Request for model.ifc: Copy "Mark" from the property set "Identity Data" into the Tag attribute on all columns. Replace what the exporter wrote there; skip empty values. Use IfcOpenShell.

First a look at what the model holds.

```python
import ifcopenshell
import ifcopenshell.util.element

model = ifcopenshell.open("model.ifc")
print(model.schema)
columns = model.by_type("IfcColumn")
print(len(columns), "columns")
for e in columns[:8]:
    source = ifcopenshell.util.element.get_pset(e, "Identity Data", "Mark")
    target = e.Tag
    print(e.id(), repr(source), repr(target), sep=" | ")
```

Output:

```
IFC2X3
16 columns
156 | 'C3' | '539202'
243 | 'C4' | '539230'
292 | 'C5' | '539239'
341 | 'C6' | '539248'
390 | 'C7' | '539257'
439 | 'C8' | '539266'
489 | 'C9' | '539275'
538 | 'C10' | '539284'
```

```python
import ifcopenshell
import ifcopenshell.util.element

model = ifcopenshell.open("model.ifc")

count = 0
for e in model.by_type("IfcColumn"):
    value = ifcopenshell.util.element.get_pset(e, "Identity Data", "Mark")
    current = e.Tag
    if not value or not value.strip() or current == value:
        continue
    e.Tag = value
    count += 1

print(count, "columns updated")

model.write("model_v2.ifc")
```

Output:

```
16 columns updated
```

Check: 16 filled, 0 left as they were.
